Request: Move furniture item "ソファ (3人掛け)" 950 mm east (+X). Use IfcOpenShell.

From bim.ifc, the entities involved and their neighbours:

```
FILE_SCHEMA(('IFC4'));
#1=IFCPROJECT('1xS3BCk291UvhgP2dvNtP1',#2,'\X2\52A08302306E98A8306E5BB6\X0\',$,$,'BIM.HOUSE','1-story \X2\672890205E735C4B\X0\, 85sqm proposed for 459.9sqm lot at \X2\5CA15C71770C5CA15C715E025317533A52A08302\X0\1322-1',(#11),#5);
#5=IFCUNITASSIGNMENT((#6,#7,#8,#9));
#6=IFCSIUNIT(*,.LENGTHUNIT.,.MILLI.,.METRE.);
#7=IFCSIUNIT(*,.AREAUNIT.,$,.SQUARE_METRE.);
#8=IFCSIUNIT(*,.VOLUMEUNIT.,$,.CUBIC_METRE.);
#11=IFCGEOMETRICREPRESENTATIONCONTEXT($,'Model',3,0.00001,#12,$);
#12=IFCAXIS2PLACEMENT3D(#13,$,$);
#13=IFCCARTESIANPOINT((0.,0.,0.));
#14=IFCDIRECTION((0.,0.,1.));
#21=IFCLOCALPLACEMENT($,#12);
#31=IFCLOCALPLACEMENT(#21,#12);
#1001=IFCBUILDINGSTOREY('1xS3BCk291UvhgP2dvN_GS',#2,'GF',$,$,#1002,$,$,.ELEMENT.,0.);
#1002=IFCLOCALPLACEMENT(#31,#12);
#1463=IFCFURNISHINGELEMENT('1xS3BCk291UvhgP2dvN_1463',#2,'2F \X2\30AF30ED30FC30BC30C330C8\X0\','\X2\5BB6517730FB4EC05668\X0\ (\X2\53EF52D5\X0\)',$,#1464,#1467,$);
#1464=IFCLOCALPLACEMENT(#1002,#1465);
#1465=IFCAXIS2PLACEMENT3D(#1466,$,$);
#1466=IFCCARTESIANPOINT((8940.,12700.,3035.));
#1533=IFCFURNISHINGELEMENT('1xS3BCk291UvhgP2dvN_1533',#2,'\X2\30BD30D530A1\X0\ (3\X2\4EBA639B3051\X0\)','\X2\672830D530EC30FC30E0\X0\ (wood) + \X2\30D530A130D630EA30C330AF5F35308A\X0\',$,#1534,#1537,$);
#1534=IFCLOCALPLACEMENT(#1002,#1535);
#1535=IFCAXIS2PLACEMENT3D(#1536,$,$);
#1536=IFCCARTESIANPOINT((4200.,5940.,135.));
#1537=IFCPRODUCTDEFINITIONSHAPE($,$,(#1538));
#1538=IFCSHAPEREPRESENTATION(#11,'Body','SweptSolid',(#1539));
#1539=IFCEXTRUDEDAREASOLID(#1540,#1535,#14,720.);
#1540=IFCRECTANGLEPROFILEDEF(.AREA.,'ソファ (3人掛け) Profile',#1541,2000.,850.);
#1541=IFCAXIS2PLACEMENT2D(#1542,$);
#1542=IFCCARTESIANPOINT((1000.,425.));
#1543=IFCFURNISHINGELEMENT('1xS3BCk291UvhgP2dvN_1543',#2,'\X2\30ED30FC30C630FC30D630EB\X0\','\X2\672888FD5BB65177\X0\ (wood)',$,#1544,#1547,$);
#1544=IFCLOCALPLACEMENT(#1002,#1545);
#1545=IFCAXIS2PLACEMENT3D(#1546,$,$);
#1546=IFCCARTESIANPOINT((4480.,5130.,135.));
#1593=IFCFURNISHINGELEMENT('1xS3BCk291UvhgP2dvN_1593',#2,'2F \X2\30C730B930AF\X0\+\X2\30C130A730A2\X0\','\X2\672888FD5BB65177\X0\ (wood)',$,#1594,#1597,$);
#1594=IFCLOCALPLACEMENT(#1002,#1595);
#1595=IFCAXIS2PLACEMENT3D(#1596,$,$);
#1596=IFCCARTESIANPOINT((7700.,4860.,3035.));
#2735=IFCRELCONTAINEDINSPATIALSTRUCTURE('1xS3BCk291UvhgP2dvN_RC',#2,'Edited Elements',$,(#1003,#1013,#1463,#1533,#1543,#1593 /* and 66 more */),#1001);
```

```python
import ifcopenshell
import ifcopenshell.api.geometry
import ifcopenshell.util.placement

model = ifcopenshell.open("bim.ifc")

item = model.by_guid("1xS3BCk291UvhgP2dvN_1533")
matrix = ifcopenshell.util.placement.get_local_placement(item.ObjectPlacement)
matrix[0, 3] += 950.0
ifcopenshell.api.geometry.edit_object_placement(model, product=item, matrix=matrix, is_si=False)

print(ifcopenshell.util.placement.get_local_placement(item.ObjectPlacement).round(3) + 0.0)

model.write("bim_edited.ifc")
```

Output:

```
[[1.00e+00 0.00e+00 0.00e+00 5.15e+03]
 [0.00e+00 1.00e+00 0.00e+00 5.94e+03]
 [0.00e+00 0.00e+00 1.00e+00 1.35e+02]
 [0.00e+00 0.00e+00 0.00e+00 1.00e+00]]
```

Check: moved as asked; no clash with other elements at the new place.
